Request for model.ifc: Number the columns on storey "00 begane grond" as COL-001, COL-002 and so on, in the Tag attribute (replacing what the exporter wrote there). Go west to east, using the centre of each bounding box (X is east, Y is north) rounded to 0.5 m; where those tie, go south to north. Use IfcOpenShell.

First a look at what the model holds.

```python
import ifcopenshell
import ifcopenshell.util.element
import ifcopenshell.util.placement

model = ifcopenshell.open("model.ifc")
print(model.schema)
storey = next(s for s in model.by_type("IfcBuildingStorey") if s.Name == "00 begane grond")
columns = [e for e in ifcopenshell.util.element.get_decomposition(storey) if e.is_a("IfcColumn")]
for e in sorted(columns, key=lambda e: e.id()):
    origin = ifcopenshell.util.placement.get_local_placement(e.ObjectPlacement)[:3, 3]
    print(e.id(), e.Tag, e.Name, origin.round(2) + 0.0, sep=" | ")
```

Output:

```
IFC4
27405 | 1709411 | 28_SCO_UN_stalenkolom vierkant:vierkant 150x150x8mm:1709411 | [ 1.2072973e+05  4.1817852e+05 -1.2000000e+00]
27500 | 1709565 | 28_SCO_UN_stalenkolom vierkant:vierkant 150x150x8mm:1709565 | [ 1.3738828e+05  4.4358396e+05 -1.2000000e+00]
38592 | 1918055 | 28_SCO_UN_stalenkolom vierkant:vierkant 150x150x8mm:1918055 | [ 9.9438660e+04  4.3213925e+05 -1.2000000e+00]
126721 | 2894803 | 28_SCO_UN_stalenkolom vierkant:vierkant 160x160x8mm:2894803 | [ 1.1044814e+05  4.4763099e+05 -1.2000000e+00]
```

```python
import ifcopenshell
import ifcopenshell.geom
import ifcopenshell.util.element
import ifcopenshell.util.shape

model = ifcopenshell.open("model.ifc")
settings = ifcopenshell.geom.settings()
settings.set("use-world-coords", True)


def centre(element):
    shape = ifcopenshell.geom.create_shape(settings, element)
    return ifcopenshell.util.shape.get_bbox_centroid(shape.geometry)


storey = next(s for s in model.by_type("IfcBuildingStorey") if s.Name == "00 begane grond")
columns = [e for e in ifcopenshell.util.element.get_decomposition(storey) if e.is_a("IfcColumn")]

# Insertion points can sit at a corner or the storey origin, so sort by the geometry (in metres).
centres = {e: centre(e) for e in columns}
columns.sort(key=lambda e: (round(centres[e][0] / 0.5), centres[e][1]))

for i, e in enumerate(columns, start=1):
    number = f"COL-0{i:02d}"
    e.Tag = number
    print(e.id(), number)

model.write("model_edited.ifc")
```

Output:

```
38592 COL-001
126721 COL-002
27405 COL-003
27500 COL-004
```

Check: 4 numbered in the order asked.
